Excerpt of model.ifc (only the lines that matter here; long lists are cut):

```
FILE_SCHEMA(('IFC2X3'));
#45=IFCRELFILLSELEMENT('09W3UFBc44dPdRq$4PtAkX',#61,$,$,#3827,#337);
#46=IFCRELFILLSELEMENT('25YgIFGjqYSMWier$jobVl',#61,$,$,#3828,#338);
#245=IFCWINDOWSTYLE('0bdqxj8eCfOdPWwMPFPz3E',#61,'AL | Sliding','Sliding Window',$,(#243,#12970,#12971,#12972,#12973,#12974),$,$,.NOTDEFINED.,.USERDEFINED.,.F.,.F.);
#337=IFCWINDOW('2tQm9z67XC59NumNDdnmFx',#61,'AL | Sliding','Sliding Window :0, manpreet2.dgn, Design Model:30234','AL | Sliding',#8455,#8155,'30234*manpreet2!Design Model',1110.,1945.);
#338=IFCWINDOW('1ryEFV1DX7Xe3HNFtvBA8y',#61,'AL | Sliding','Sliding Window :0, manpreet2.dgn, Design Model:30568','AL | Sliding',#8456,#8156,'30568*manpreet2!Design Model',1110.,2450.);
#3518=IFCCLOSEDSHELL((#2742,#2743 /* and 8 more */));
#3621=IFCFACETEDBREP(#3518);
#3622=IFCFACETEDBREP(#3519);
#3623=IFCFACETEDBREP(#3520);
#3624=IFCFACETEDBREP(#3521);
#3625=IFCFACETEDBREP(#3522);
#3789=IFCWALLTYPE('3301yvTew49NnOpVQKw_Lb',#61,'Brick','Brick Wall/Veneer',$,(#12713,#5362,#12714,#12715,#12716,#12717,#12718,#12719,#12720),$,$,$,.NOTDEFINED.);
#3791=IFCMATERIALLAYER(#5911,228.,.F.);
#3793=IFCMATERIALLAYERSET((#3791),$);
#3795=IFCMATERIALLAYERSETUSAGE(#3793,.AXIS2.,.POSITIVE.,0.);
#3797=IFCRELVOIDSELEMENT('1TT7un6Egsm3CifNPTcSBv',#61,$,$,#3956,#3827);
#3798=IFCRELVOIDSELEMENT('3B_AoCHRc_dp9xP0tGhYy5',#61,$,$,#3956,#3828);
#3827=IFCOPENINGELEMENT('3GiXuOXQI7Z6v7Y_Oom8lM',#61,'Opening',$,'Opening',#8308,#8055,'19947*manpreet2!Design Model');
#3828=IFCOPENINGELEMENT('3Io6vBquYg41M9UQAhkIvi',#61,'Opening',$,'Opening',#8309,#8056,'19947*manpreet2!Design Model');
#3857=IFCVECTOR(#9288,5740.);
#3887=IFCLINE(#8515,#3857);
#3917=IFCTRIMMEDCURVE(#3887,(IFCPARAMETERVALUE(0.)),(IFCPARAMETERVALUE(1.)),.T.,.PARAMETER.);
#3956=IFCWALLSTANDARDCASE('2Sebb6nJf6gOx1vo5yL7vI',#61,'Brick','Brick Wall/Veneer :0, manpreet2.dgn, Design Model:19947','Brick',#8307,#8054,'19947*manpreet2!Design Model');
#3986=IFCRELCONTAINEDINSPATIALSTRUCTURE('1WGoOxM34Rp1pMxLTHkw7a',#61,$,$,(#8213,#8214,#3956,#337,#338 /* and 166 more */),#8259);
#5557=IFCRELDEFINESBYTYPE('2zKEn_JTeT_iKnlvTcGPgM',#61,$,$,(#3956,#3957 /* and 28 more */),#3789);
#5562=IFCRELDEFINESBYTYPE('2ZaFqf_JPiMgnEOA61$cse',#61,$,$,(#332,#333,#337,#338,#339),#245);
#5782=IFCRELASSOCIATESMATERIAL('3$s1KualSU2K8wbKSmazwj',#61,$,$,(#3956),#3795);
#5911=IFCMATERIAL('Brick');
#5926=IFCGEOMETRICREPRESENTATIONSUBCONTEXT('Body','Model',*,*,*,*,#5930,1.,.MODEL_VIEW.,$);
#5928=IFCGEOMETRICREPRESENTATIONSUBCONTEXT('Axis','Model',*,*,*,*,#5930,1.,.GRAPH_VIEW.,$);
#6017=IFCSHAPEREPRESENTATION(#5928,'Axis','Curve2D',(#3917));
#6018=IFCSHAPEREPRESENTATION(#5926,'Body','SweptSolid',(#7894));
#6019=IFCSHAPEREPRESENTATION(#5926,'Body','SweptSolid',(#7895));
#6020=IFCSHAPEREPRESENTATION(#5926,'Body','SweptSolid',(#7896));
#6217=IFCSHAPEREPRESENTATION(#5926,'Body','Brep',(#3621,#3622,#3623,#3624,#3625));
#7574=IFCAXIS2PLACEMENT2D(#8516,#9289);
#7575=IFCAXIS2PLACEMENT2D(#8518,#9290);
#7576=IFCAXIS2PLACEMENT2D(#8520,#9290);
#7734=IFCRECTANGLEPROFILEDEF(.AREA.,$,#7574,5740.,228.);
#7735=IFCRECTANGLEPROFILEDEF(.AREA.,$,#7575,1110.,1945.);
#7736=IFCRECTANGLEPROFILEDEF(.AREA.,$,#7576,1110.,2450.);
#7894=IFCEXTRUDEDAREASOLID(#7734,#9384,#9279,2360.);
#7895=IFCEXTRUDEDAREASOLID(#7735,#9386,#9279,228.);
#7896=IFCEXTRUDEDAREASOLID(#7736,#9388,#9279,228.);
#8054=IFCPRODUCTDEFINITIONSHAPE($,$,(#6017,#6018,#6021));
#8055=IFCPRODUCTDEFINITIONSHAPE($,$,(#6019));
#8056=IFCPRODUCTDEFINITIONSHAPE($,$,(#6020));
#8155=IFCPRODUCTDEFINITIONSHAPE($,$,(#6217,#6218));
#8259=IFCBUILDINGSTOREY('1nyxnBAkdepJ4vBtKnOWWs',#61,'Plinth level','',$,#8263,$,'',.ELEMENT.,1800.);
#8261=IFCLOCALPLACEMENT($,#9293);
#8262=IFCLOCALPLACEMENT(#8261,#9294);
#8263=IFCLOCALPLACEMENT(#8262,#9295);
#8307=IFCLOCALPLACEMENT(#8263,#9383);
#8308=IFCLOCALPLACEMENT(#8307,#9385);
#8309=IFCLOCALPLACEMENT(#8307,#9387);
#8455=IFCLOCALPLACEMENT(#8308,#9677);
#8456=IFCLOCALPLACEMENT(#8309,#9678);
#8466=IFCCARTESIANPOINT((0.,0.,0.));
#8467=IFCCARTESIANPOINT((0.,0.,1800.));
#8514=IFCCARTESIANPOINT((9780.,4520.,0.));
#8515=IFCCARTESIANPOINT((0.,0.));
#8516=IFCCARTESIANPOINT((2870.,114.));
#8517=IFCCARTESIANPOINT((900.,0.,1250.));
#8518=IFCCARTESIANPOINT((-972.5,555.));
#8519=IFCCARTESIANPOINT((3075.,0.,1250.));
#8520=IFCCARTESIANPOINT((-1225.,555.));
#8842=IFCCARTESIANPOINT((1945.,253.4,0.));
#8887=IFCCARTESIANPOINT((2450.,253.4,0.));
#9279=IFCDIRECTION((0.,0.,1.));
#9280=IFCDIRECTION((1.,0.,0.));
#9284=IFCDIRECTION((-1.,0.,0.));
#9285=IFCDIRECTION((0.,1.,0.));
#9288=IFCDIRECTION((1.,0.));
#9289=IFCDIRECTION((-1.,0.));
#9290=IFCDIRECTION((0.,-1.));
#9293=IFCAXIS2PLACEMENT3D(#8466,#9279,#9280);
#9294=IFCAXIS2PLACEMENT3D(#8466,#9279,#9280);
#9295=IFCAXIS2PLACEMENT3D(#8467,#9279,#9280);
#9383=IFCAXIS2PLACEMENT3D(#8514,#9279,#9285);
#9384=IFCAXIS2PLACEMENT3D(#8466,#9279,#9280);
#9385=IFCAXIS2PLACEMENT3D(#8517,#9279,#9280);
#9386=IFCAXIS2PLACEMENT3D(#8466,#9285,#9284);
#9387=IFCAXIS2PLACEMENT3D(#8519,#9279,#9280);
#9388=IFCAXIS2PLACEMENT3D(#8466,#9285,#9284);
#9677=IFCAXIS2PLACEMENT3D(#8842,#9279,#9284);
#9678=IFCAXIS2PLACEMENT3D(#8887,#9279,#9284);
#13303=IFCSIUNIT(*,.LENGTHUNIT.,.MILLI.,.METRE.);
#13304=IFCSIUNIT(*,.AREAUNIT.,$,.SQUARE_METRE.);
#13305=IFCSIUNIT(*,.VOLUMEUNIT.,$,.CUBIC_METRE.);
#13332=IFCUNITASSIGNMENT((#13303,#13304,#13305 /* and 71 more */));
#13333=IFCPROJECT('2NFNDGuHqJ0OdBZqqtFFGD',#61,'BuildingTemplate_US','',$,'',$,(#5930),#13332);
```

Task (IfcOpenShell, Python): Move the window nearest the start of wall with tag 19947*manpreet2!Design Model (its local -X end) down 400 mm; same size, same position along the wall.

```python
import numpy as np
import ifcopenshell
import ifcopenshell.api.geometry
import ifcopenshell.util.placement
import ifcopenshell.util.unit

model = ifcopenshell.open("model.ifc")
unit_scale = ifcopenshell.util.unit.calculate_unit_scale(model)

window = model.by_guid("2tQm9z67XC59NumNDdnmFx")
opening = window.FillsVoids[0].RelatingOpeningElement
dz = -0.4 / unit_scale

shift = np.array([0.0, 0.0, dz])
# The window is placed relative to its opening, so it follows when the opening moves.
matrix = ifcopenshell.util.placement.get_local_placement(opening.ObjectPlacement)
matrix[:3, 3] += shift
ifcopenshell.api.geometry.edit_object_placement(
    model, product=opening, matrix=matrix, is_si=False, should_transform_children=True
)

print(f"moved by {dz * unit_scale:+.3f} m")

model.write("model-out.ifc")
```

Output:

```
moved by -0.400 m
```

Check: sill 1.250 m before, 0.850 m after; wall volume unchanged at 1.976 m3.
